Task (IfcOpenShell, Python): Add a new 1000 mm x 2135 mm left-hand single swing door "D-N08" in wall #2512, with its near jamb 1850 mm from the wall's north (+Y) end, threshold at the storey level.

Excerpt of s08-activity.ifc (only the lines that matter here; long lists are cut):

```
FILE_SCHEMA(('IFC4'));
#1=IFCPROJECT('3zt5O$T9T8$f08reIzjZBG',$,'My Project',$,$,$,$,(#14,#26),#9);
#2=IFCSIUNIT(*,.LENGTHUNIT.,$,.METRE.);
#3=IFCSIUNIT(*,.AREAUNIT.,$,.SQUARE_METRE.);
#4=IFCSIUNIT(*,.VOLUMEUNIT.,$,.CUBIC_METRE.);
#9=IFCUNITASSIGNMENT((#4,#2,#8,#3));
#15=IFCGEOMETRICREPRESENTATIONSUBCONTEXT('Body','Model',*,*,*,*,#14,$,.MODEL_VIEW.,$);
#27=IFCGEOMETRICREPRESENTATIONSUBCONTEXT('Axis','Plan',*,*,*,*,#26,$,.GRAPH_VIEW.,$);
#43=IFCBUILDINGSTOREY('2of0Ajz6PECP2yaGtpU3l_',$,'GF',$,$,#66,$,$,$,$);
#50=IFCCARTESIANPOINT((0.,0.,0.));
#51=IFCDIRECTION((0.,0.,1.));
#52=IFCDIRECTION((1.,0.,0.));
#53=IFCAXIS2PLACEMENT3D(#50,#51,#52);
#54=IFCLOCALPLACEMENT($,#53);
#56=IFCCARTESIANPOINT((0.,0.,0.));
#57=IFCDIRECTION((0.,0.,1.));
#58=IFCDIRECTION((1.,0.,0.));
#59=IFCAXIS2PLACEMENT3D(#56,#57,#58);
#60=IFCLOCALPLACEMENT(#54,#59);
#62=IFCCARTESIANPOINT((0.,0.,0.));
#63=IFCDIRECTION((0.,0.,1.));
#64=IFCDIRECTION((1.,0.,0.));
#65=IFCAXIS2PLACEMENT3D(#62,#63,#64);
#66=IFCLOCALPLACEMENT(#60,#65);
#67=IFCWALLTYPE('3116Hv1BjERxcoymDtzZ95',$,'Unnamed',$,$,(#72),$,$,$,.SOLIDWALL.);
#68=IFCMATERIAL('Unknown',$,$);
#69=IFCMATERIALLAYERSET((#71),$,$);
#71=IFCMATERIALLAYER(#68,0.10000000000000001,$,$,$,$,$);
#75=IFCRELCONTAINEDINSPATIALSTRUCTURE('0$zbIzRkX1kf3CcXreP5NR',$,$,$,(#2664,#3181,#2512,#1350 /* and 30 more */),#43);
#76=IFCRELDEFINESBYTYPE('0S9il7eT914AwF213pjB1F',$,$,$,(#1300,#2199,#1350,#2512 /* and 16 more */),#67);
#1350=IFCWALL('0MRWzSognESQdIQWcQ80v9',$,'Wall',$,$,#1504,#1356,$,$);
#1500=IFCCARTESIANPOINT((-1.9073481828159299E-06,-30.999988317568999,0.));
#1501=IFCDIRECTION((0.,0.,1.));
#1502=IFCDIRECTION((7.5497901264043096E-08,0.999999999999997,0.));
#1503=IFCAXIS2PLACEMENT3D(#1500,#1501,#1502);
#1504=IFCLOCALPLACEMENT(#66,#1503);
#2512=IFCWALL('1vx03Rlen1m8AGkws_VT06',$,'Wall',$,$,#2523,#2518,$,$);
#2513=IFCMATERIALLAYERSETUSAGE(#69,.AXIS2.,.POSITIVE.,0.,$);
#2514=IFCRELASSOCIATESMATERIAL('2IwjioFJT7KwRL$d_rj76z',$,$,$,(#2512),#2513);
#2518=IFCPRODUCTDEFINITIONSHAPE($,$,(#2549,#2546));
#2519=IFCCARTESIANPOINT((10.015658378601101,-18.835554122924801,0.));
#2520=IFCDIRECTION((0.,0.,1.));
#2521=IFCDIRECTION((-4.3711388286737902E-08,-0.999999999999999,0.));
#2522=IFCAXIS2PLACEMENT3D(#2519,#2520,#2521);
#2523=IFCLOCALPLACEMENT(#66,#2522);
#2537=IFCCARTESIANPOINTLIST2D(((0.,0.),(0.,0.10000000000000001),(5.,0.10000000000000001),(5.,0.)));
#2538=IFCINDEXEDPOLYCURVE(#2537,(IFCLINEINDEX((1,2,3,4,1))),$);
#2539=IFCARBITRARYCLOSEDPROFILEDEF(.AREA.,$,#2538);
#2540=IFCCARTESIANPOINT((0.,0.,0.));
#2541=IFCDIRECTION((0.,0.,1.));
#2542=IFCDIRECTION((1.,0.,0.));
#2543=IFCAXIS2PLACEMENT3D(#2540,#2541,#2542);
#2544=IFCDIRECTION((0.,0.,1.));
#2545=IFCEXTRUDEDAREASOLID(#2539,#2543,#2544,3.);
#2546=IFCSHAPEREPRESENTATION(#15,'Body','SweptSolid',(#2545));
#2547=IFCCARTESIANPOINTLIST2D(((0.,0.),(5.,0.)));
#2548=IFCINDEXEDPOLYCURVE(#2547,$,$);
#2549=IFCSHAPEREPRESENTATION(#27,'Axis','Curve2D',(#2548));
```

```python
import numpy as np
import ifcopenshell
import ifcopenshell.api.feature
import ifcopenshell.api.geometry
import ifcopenshell.api.root
import ifcopenshell.api.spatial
import ifcopenshell.geom
import ifcopenshell.util.element
import ifcopenshell.util.placement
import ifcopenshell.util.representation
import ifcopenshell.util.shape
import ifcopenshell.util.unit

model = ifcopenshell.open("s08-activity.ifc")
unit_scale = ifcopenshell.util.unit.calculate_unit_scale(model)
settings = ifcopenshell.geom.settings()


def volume(element):
    """Net volume in cubic metres, openings subtracted."""
    shape = ifcopenshell.geom.create_shape(settings, element)
    return ifcopenshell.util.shape.get_volume(shape.geometry)


wall = model.by_id(2512)
storey = ifcopenshell.util.element.get_container(wall, ifc_class="IfcBuildingStorey")
context = ifcopenshell.util.representation.get_context(model, "Model", "Body", "MODEL_VIEW")
before = volume(wall)

width, height, from_end, sill = 1, 2.135, 1.85, 0.0  # metres

# The wall runs along its own X axis, and the end named is its -X end.
wall_shape = ifcopenshell.geom.create_shape(settings, wall)
x, y, z = ifcopenshell.util.shape.get_vertices(wall_shape.geometry).T
start = x.min() + from_end
face, thickness = float(y.min()), float(y.max() - y.min())
wall_matrix = ifcopenshell.util.placement.get_local_placement(wall.ObjectPlacement)
level = ifcopenshell.util.placement.get_local_placement(storey.ObjectPlacement)[2, 3]


def in_wall(x, y):
    """Placement at x, y metres in the wall's axes, at sill height."""
    matrix = wall_matrix.copy()
    matrix[:, 3] = wall_matrix @ np.array([x / unit_scale, y / unit_scale, 0.0, 1.0])
    matrix[2, 3] = level + sill / unit_scale
    return matrix


# Opening: a box that overshoots both wall faces by 50 mm.
opening = ifcopenshell.api.root.create_entity(model, ifc_class="IfcOpeningElement", predefined_type="OPENING")
box = ifcopenshell.api.geometry.add_wall_representation(
    model, context=context, length=width, height=height, thickness=thickness + 0.1
)
ifcopenshell.api.geometry.assign_representation(model, product=opening, representation=box)
ifcopenshell.api.geometry.edit_object_placement(model, product=opening, matrix=in_wall(start, face - 0.05), is_si=False)
ifcopenshell.api.feature.add_feature(model, feature=opening, element=wall)

door = ifcopenshell.api.root.create_entity(model, ifc_class="IfcDoor", name="D-N08", predefined_type="DOOR")
door.OverallWidth, door.OverallHeight = width / unit_scale, height / unit_scale
door.OperationType = "SINGLE_SWING_LEFT"
body = ifcopenshell.api.geometry.add_door_representation(
    model,
    context=context,
    overall_width=door.OverallWidth,
    overall_height=door.OverallHeight,
    operation_type="SINGLE_SWING_LEFT",
    lining_properties={"LiningDepth": thickness / unit_scale, "ThresholdDepth": thickness / unit_scale},
)
ifcopenshell.api.geometry.assign_representation(model, product=door, representation=body)
ifcopenshell.api.spatial.assign_container(model, products=[door], relating_structure=storey)
ifcopenshell.api.feature.add_filling(model, opening=opening, element=door)

# The lining spans the wall, so the door starts at the wall face.
ifcopenshell.api.geometry.edit_object_placement(model, product=door, matrix=in_wall(start, face), is_si=False)

after = volume(wall)

print(f"wall volume {before:.3f} -> {after:.3f} m3")

model.write("s08-activity_v2.ifc")
```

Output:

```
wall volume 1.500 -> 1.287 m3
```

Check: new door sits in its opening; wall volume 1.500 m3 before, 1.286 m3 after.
